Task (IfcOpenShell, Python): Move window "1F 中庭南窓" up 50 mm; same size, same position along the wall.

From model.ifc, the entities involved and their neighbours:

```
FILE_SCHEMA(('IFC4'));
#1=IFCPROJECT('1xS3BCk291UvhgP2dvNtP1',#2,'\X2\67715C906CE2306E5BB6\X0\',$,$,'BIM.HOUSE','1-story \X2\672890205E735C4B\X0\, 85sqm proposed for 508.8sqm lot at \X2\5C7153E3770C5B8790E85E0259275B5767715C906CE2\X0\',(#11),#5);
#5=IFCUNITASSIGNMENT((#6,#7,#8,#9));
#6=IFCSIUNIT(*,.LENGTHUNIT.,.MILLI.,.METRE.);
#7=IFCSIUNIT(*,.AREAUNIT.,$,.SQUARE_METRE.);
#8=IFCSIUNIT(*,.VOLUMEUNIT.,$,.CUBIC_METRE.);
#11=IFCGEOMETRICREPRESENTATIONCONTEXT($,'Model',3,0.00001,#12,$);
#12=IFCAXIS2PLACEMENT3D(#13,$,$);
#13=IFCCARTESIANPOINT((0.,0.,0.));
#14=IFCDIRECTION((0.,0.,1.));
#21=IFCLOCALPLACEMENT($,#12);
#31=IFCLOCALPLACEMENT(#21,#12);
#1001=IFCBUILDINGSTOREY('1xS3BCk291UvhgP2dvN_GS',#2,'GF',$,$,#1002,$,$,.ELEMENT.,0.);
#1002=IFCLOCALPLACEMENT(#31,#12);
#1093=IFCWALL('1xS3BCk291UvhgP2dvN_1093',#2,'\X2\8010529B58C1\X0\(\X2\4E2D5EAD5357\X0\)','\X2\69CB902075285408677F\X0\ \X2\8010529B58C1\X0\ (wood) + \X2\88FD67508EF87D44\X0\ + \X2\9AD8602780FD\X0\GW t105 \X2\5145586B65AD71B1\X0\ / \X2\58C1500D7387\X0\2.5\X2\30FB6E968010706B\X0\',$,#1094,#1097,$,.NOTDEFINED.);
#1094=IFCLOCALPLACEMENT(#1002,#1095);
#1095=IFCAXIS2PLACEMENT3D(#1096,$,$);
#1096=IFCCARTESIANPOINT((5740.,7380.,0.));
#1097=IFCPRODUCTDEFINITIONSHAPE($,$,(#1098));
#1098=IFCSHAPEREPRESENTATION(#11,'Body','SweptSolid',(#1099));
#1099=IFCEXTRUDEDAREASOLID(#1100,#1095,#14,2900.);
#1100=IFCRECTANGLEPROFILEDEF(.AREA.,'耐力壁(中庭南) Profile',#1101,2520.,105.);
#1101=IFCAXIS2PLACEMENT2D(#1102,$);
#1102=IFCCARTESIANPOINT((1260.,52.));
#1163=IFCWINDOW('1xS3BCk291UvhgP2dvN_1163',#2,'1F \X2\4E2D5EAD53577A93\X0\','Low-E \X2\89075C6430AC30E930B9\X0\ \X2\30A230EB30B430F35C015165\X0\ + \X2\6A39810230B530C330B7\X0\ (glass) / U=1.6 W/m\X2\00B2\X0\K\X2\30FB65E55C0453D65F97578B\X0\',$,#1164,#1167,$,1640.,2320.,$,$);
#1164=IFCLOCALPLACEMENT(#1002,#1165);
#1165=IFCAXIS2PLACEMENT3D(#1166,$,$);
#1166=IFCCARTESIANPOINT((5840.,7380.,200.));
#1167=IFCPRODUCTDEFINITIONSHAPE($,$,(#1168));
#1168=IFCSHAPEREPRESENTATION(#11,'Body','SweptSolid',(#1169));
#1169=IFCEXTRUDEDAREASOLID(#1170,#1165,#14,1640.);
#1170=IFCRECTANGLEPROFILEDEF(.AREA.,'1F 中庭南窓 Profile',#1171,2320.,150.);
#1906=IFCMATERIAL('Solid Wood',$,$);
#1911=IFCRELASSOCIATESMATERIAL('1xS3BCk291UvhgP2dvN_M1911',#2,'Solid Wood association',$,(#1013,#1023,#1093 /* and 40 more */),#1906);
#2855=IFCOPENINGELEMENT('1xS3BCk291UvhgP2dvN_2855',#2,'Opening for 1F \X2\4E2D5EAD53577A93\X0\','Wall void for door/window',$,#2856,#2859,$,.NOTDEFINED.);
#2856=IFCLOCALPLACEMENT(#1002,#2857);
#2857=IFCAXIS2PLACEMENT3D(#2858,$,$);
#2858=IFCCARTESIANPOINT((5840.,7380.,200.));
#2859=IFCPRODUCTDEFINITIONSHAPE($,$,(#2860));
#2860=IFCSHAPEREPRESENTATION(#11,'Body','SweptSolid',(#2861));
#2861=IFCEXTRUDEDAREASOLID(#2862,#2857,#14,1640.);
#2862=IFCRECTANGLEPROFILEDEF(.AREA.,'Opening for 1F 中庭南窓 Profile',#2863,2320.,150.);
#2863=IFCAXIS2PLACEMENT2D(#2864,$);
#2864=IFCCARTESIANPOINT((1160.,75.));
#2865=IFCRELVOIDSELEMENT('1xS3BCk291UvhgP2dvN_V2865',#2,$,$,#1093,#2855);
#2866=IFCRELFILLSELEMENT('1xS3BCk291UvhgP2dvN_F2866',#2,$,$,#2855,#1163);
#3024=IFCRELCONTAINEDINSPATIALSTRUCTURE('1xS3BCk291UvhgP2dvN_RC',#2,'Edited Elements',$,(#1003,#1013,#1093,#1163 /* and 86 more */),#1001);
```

```python
import numpy as np
import ifcopenshell
import ifcopenshell.api.geometry
import ifcopenshell.util.placement
import ifcopenshell.util.unit

model = ifcopenshell.open("model.ifc")
unit_scale = ifcopenshell.util.unit.calculate_unit_scale(model)

window = model.by_id(1163)
opening = window.FillsVoids[0].RelatingOpeningElement
dz = 0.05 / unit_scale

shift = np.array([0.0, 0.0, dz])
# The window is not placed relative to its opening, so move both.
for product in (opening, window):
    matrix = ifcopenshell.util.placement.get_local_placement(product.ObjectPlacement)
    matrix[:3, 3] += shift
    ifcopenshell.api.geometry.edit_object_placement(model, product=product, matrix=matrix, is_si=False)

print(f"moved by {dz * unit_scale:+.3f} m")

model.write("model_v2.ifc")
```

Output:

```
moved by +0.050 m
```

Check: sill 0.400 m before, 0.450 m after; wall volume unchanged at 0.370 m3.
